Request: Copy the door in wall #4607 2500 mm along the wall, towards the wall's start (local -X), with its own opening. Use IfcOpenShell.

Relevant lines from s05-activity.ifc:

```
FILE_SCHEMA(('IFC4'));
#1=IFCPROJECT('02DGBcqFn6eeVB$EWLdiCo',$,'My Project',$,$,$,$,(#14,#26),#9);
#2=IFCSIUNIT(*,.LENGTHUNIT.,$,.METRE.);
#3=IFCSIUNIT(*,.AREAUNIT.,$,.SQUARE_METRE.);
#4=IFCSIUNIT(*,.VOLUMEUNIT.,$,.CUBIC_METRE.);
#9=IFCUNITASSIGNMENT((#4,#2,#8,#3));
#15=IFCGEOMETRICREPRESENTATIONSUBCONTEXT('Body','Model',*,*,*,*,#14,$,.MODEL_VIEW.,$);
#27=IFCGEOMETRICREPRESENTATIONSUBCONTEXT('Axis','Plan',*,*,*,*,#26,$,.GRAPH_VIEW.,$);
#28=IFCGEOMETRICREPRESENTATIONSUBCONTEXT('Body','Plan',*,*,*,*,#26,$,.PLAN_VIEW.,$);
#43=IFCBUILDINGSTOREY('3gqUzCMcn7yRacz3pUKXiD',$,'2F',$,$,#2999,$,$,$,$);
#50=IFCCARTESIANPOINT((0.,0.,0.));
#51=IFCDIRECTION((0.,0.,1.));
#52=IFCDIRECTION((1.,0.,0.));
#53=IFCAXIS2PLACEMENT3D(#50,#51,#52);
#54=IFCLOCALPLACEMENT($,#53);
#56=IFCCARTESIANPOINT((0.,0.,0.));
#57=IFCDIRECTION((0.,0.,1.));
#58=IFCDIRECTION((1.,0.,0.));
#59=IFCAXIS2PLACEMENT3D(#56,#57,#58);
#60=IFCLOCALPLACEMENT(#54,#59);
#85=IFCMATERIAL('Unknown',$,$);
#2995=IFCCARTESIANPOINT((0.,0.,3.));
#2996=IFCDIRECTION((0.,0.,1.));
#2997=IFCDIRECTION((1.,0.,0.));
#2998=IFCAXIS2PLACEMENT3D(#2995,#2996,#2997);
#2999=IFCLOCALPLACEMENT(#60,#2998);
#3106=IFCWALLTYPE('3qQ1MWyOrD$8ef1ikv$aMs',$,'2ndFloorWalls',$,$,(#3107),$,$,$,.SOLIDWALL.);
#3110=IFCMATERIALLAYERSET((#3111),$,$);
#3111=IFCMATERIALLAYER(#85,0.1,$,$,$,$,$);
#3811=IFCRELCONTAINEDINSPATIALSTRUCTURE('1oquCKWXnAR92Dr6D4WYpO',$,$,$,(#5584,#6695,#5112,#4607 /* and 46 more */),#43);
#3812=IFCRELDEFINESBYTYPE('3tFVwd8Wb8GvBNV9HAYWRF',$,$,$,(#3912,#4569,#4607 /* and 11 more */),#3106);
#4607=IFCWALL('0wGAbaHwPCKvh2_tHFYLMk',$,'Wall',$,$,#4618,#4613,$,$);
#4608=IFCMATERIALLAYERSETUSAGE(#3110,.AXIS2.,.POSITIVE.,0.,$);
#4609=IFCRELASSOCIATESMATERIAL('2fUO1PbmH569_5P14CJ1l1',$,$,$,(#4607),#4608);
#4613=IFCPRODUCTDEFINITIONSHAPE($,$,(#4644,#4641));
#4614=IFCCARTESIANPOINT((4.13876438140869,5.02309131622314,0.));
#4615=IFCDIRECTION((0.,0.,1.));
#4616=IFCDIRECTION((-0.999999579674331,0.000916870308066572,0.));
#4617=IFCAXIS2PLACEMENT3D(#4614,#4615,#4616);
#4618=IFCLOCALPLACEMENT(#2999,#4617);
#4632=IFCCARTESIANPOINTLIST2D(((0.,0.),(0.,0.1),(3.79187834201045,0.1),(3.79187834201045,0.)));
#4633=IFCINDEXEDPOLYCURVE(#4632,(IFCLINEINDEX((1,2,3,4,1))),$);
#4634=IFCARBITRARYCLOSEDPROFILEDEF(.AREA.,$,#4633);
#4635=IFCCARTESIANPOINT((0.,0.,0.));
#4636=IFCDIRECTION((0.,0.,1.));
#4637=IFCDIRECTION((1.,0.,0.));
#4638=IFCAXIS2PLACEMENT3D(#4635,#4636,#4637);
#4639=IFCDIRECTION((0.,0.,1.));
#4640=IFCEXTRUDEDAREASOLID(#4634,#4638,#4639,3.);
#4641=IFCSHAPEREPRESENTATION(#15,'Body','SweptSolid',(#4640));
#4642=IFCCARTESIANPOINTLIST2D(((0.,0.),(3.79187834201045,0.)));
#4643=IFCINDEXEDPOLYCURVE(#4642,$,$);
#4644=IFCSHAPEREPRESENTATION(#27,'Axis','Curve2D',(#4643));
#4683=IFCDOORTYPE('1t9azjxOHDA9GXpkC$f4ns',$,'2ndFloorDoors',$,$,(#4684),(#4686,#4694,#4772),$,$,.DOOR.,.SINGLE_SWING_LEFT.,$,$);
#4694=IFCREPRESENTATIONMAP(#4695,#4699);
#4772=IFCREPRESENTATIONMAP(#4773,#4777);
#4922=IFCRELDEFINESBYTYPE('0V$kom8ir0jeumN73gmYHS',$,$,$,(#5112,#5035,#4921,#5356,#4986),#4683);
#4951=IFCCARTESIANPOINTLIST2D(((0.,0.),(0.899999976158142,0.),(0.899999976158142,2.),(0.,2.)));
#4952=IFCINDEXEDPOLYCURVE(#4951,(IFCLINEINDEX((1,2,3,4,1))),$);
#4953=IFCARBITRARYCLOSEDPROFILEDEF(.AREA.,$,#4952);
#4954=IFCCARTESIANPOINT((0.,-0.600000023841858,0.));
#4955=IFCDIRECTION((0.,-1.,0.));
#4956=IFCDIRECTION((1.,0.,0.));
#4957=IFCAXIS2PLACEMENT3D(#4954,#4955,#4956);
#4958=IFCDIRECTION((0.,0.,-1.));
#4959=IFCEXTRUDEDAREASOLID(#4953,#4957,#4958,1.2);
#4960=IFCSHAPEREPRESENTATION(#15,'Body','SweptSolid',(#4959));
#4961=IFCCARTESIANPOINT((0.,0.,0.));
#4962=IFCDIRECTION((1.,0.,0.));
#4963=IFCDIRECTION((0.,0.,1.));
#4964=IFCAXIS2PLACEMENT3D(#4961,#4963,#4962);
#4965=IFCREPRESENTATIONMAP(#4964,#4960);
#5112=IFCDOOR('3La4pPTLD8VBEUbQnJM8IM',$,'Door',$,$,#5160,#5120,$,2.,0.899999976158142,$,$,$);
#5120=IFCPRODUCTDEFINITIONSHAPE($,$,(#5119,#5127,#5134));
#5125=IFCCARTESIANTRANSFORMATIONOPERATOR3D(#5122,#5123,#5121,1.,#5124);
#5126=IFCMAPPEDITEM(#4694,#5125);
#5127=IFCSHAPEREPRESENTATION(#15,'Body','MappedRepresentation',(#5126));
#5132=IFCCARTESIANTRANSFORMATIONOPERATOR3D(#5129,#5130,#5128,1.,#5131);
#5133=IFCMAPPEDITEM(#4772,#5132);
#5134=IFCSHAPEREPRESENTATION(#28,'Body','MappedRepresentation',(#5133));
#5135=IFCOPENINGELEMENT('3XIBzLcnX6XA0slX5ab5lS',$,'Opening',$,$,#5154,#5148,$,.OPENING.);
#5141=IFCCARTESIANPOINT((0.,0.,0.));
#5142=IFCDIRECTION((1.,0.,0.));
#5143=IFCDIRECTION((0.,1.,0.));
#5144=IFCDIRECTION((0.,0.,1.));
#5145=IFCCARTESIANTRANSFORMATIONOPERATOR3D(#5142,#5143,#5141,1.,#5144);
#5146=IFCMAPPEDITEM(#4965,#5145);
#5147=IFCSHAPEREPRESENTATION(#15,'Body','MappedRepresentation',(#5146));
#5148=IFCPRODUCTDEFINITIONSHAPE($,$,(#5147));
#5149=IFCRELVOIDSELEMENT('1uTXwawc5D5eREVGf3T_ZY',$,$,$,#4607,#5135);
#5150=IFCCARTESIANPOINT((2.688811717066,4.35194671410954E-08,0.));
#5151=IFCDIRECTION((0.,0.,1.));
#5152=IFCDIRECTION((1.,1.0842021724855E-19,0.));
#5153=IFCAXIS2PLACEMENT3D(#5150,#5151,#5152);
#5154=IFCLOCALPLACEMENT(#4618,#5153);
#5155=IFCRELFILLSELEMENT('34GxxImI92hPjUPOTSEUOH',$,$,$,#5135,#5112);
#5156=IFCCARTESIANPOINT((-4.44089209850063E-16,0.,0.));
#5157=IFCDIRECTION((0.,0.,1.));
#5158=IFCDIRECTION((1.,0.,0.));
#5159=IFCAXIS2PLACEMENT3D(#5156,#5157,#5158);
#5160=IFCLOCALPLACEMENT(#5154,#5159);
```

```python
import ifcopenshell
import ifcopenshell.api.feature
import ifcopenshell.api.geometry
import ifcopenshell.api.root
import ifcopenshell.geom
import ifcopenshell.util.element
import ifcopenshell.util.placement
import ifcopenshell.util.shape
import ifcopenshell.util.unit

model = ifcopenshell.open("s05-activity.ifc")
unit_scale = ifcopenshell.util.unit.calculate_unit_scale(model)
settings = ifcopenshell.geom.settings()


def volume(element):
    """Net volume in cubic metres, openings subtracted."""
    shape = ifcopenshell.geom.create_shape(settings, element)
    return ifcopenshell.util.shape.get_volume(shape.geometry)


door = model.by_id(5112)
opening = door.FillsVoids[0].RelatingOpeningElement
wall = opening.VoidsElements[0].RelatingBuildingElement
before = volume(wall)
shift = ifcopenshell.util.placement.get_local_placement(wall.ObjectPlacement)[:3, 0] * -2.5 / unit_scale

# copy_class copies the void relationship, type, container and properties, but no geometry.
new_opening = ifcopenshell.api.root.copy_class(model, product=opening)
new_opening.Representation = ifcopenshell.util.element.copy_deep(
    model, opening.Representation, exclude=["IfcGeometricRepresentationContext", "IfcRepresentationMap"]
)
new_door = ifcopenshell.api.root.copy_class(model, product=door)
new_door.Representation = ifcopenshell.util.element.copy_deep(
    model, door.Representation, exclude=["IfcGeometricRepresentationContext", "IfcRepresentationMap"]
)
ifcopenshell.api.feature.add_filling(model, opening=new_opening, element=new_door)

for old, new in ((opening, new_opening), (door, new_door)):
    matrix = ifcopenshell.util.placement.get_local_placement(old.ObjectPlacement)
    matrix[:3, 3] += shift
    ifcopenshell.api.geometry.edit_object_placement(model, product=new, matrix=matrix, is_si=False)

after = volume(wall)

print(f"wall volume {before:.3f} -> {after:.3f} m3")

model.write("s05-activity_edited.ifc")
```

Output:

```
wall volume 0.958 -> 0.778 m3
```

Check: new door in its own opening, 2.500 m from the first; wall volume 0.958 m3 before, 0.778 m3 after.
